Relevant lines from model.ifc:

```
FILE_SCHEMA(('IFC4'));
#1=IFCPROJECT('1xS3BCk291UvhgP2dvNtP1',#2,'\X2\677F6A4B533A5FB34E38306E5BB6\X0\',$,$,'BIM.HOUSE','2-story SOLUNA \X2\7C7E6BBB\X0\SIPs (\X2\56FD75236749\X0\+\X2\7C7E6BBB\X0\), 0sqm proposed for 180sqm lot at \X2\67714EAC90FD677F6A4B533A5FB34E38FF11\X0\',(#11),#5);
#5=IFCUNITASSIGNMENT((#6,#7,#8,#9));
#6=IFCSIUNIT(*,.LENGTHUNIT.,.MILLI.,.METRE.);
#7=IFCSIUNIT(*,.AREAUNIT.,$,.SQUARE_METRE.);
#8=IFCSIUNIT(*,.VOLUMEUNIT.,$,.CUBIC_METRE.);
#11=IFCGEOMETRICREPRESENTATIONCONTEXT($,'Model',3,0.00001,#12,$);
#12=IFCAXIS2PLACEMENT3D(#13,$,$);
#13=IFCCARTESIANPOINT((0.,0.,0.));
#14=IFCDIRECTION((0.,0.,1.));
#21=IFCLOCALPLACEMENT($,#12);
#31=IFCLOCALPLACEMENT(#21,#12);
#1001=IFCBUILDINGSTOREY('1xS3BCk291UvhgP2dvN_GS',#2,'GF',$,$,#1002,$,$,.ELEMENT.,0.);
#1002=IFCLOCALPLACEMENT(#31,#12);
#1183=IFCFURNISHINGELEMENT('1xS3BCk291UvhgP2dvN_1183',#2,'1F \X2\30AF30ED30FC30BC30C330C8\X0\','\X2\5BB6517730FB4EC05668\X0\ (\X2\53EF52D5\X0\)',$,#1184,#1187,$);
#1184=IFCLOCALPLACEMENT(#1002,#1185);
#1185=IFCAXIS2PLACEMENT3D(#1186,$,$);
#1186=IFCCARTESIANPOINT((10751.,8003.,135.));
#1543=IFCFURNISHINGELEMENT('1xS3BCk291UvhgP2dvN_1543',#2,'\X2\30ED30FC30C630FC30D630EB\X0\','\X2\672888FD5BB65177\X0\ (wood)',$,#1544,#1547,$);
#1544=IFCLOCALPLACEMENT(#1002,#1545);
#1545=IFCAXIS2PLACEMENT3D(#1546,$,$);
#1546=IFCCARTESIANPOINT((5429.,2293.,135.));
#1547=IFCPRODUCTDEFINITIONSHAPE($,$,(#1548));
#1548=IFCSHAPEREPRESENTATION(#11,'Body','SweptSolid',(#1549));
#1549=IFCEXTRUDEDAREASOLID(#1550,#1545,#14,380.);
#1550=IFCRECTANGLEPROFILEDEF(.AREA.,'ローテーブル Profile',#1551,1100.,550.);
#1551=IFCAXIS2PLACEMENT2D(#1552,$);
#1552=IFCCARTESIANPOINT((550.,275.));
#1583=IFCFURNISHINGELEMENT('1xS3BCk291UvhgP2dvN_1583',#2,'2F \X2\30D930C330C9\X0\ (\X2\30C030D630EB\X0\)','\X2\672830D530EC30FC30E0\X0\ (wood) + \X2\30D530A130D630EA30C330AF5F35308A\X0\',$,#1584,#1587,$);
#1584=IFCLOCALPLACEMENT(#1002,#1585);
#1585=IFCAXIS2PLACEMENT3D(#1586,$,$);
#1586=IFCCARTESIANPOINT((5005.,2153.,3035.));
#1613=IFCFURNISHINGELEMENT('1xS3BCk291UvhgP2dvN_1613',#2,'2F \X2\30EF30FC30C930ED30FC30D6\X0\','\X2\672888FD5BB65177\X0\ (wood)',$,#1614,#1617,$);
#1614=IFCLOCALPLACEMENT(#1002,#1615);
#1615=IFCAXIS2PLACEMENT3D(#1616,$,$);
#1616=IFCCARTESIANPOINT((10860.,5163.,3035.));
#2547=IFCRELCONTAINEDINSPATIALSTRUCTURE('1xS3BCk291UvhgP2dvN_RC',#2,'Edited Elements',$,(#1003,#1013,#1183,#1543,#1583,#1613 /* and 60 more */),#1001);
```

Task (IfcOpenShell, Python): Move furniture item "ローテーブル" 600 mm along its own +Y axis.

```python
import ifcopenshell
import ifcopenshell.api.geometry
import ifcopenshell.util.placement

model = ifcopenshell.open("model.ifc")

item = model.by_guid("1xS3BCk291UvhgP2dvN_1543")
matrix = ifcopenshell.util.placement.get_local_placement(item.ObjectPlacement)
matrix[:3, 3] += matrix[:3, 1] * 600.0
ifcopenshell.api.geometry.edit_object_placement(model, product=item, matrix=matrix, is_si=False)

print(ifcopenshell.util.placement.get_local_placement(item.ObjectPlacement).round(3) + 0.0)

model.write("model_updated.ifc")
```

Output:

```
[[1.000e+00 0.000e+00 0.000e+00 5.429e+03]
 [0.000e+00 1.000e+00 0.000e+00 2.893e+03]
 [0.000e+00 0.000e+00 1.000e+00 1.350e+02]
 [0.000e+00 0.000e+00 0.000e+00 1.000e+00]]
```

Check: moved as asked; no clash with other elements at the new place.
